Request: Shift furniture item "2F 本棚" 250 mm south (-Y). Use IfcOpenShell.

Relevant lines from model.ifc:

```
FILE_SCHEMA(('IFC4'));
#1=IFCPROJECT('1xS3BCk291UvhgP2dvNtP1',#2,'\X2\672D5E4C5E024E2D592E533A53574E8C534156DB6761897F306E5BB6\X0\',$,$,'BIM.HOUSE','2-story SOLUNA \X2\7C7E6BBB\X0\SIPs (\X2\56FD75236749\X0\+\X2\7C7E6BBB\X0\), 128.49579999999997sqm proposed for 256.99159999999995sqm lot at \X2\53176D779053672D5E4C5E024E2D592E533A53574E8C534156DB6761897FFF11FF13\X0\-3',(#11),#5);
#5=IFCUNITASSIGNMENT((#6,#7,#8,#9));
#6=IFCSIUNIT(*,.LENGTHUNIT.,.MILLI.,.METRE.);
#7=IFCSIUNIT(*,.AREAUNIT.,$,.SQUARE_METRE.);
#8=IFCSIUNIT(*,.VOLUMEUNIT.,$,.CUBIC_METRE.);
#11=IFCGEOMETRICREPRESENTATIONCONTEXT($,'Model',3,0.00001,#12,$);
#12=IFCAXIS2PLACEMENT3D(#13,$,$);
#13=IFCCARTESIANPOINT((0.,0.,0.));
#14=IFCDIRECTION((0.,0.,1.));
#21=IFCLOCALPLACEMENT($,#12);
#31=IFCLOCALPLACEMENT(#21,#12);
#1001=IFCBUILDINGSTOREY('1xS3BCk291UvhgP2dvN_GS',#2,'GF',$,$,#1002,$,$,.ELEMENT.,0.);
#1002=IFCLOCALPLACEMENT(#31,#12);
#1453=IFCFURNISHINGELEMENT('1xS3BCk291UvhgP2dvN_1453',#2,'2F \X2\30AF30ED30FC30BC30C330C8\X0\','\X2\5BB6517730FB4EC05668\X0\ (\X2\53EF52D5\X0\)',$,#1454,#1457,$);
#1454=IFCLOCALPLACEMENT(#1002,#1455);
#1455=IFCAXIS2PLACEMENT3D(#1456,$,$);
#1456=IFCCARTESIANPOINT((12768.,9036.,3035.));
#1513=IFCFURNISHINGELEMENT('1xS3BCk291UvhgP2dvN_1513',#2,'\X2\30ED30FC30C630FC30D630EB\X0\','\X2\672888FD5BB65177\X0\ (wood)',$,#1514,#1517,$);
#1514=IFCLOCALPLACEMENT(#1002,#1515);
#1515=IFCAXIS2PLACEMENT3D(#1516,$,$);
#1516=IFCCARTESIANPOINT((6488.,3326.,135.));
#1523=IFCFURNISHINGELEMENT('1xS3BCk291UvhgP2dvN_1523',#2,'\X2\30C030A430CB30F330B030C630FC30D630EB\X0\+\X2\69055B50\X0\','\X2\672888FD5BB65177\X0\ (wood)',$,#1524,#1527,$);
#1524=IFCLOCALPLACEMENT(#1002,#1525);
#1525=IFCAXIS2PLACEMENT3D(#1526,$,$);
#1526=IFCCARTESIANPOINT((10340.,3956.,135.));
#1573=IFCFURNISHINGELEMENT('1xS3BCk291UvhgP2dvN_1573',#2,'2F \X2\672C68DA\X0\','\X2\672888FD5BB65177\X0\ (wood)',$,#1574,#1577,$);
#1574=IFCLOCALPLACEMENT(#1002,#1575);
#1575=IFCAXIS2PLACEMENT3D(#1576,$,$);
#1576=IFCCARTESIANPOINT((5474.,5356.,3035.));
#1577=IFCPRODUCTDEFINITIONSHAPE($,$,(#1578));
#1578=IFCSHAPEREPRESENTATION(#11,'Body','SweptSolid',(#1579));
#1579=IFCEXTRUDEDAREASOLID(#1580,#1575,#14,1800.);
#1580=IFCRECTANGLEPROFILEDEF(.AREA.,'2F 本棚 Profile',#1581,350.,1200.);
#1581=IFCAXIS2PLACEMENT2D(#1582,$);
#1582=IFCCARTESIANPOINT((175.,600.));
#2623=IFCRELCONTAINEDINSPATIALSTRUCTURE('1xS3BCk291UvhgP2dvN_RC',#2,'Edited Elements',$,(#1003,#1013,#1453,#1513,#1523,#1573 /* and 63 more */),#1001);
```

```python
import ifcopenshell
import ifcopenshell.api.geometry
import ifcopenshell.util.placement
import ifcopenshell.util.unit

model = ifcopenshell.open("model.ifc")
unit_scale = ifcopenshell.util.unit.calculate_unit_scale(model)

item = model.by_id(1573)
matrix = ifcopenshell.util.placement.get_local_placement(item.ObjectPlacement)
matrix[1, 3] -= 0.25 / unit_scale
ifcopenshell.api.geometry.edit_object_placement(model, product=item, matrix=matrix, is_si=False)

print(ifcopenshell.util.placement.get_local_placement(item.ObjectPlacement).round(3) + 0.0)

model.write("model_v2.ifc")
```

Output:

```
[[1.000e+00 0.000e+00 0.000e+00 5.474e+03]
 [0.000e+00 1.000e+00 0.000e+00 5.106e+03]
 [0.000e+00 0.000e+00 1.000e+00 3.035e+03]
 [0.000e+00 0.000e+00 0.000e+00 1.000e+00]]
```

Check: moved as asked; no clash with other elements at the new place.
